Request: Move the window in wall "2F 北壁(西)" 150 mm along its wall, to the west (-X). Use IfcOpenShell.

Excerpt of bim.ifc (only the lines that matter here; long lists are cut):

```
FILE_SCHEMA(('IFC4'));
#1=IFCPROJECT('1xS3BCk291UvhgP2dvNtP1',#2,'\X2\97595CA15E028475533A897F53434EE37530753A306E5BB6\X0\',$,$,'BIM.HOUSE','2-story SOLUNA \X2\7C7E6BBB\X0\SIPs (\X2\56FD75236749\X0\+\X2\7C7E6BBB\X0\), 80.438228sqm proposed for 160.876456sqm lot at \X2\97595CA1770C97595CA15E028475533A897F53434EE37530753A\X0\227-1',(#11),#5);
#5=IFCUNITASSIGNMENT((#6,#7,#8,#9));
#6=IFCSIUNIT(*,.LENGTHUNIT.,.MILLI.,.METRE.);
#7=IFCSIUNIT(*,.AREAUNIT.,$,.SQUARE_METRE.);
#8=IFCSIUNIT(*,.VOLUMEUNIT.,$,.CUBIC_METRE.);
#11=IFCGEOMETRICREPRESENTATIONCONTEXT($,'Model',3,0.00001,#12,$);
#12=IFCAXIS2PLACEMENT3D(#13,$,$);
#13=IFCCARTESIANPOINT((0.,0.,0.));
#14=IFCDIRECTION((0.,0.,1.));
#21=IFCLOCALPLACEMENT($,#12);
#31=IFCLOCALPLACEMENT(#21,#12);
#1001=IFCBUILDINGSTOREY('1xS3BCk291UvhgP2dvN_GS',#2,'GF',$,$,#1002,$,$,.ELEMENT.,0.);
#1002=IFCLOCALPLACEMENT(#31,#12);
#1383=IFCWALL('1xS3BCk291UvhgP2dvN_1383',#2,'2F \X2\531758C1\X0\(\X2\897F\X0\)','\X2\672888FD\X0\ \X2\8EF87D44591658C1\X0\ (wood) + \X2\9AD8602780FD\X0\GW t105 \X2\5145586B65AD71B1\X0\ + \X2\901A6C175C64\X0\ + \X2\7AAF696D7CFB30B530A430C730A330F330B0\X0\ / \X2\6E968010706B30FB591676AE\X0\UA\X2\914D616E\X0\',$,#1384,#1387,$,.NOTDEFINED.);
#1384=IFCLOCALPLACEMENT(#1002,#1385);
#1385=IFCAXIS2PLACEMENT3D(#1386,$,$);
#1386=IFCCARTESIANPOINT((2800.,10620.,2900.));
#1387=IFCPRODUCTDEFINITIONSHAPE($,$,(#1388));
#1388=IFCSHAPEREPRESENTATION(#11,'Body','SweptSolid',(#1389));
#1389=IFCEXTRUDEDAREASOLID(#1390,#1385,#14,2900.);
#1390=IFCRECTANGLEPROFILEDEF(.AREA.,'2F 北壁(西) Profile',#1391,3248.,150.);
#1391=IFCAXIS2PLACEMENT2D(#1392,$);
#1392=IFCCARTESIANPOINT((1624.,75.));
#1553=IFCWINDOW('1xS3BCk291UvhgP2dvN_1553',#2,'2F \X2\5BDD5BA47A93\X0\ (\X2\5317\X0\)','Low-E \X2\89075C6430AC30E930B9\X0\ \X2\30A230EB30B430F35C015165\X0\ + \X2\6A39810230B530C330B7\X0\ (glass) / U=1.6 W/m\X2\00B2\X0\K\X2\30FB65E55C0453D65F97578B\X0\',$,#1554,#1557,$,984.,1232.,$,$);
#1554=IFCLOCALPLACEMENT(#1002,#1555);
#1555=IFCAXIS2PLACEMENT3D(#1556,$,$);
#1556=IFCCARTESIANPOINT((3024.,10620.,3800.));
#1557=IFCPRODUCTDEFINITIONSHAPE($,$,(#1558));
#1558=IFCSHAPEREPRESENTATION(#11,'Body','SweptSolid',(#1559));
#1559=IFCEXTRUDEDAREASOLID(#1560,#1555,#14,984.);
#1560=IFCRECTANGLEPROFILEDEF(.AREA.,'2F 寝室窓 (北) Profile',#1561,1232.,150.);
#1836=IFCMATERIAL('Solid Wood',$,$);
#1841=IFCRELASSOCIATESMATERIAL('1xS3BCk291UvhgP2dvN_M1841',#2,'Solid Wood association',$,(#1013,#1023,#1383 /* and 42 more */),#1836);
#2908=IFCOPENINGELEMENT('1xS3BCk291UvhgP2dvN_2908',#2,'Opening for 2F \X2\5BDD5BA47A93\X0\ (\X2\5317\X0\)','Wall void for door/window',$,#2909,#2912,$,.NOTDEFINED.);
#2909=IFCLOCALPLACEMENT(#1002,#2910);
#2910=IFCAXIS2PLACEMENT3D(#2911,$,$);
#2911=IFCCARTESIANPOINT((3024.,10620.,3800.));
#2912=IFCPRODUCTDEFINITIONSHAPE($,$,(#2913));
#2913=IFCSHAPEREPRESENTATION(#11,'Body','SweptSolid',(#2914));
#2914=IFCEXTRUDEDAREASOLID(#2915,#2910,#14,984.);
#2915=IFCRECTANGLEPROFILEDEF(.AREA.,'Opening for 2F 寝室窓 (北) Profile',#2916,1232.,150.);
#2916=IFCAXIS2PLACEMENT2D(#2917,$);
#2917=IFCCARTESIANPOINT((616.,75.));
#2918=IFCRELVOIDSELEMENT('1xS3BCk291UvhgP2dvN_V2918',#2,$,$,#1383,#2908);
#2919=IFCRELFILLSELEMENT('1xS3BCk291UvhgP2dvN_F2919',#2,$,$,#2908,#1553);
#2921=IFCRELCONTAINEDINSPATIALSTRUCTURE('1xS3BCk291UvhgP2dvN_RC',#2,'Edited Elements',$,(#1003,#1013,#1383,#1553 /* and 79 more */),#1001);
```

```python
import ifcopenshell
import ifcopenshell.api.geometry
import ifcopenshell.util.placement
import ifcopenshell.util.unit

model = ifcopenshell.open("bim.ifc")
unit_scale = ifcopenshell.util.unit.calculate_unit_scale(model)

window = model.by_guid("1xS3BCk291UvhgP2dvN_1553")
opening = window.FillsVoids[0].RelatingOpeningElement
wall = opening.VoidsElements[0].RelatingBuildingElement

wall_matrix = ifcopenshell.util.placement.get_local_placement(wall.ObjectPlacement)
shift = wall_matrix[:3, 0] * -0.15 / unit_scale
before = ifcopenshell.util.placement.get_local_placement(window.ObjectPlacement)[:3, 3].copy()

# The window is not placed relative to its opening, so move both.
for product in (opening, window):
    matrix = ifcopenshell.util.placement.get_local_placement(product.ObjectPlacement)
    matrix[:3, 3] += shift
    ifcopenshell.api.geometry.edit_object_placement(model, product=product, matrix=matrix, is_si=False)

after = ifcopenshell.util.placement.get_local_placement(window.ObjectPlacement)[:3, 3]
print("window moved by", (after - before).round(3) + 0.0)

model.write("bim_updated.ifc")
```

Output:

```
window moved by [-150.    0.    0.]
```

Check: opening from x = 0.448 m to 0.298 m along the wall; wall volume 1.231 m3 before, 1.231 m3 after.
